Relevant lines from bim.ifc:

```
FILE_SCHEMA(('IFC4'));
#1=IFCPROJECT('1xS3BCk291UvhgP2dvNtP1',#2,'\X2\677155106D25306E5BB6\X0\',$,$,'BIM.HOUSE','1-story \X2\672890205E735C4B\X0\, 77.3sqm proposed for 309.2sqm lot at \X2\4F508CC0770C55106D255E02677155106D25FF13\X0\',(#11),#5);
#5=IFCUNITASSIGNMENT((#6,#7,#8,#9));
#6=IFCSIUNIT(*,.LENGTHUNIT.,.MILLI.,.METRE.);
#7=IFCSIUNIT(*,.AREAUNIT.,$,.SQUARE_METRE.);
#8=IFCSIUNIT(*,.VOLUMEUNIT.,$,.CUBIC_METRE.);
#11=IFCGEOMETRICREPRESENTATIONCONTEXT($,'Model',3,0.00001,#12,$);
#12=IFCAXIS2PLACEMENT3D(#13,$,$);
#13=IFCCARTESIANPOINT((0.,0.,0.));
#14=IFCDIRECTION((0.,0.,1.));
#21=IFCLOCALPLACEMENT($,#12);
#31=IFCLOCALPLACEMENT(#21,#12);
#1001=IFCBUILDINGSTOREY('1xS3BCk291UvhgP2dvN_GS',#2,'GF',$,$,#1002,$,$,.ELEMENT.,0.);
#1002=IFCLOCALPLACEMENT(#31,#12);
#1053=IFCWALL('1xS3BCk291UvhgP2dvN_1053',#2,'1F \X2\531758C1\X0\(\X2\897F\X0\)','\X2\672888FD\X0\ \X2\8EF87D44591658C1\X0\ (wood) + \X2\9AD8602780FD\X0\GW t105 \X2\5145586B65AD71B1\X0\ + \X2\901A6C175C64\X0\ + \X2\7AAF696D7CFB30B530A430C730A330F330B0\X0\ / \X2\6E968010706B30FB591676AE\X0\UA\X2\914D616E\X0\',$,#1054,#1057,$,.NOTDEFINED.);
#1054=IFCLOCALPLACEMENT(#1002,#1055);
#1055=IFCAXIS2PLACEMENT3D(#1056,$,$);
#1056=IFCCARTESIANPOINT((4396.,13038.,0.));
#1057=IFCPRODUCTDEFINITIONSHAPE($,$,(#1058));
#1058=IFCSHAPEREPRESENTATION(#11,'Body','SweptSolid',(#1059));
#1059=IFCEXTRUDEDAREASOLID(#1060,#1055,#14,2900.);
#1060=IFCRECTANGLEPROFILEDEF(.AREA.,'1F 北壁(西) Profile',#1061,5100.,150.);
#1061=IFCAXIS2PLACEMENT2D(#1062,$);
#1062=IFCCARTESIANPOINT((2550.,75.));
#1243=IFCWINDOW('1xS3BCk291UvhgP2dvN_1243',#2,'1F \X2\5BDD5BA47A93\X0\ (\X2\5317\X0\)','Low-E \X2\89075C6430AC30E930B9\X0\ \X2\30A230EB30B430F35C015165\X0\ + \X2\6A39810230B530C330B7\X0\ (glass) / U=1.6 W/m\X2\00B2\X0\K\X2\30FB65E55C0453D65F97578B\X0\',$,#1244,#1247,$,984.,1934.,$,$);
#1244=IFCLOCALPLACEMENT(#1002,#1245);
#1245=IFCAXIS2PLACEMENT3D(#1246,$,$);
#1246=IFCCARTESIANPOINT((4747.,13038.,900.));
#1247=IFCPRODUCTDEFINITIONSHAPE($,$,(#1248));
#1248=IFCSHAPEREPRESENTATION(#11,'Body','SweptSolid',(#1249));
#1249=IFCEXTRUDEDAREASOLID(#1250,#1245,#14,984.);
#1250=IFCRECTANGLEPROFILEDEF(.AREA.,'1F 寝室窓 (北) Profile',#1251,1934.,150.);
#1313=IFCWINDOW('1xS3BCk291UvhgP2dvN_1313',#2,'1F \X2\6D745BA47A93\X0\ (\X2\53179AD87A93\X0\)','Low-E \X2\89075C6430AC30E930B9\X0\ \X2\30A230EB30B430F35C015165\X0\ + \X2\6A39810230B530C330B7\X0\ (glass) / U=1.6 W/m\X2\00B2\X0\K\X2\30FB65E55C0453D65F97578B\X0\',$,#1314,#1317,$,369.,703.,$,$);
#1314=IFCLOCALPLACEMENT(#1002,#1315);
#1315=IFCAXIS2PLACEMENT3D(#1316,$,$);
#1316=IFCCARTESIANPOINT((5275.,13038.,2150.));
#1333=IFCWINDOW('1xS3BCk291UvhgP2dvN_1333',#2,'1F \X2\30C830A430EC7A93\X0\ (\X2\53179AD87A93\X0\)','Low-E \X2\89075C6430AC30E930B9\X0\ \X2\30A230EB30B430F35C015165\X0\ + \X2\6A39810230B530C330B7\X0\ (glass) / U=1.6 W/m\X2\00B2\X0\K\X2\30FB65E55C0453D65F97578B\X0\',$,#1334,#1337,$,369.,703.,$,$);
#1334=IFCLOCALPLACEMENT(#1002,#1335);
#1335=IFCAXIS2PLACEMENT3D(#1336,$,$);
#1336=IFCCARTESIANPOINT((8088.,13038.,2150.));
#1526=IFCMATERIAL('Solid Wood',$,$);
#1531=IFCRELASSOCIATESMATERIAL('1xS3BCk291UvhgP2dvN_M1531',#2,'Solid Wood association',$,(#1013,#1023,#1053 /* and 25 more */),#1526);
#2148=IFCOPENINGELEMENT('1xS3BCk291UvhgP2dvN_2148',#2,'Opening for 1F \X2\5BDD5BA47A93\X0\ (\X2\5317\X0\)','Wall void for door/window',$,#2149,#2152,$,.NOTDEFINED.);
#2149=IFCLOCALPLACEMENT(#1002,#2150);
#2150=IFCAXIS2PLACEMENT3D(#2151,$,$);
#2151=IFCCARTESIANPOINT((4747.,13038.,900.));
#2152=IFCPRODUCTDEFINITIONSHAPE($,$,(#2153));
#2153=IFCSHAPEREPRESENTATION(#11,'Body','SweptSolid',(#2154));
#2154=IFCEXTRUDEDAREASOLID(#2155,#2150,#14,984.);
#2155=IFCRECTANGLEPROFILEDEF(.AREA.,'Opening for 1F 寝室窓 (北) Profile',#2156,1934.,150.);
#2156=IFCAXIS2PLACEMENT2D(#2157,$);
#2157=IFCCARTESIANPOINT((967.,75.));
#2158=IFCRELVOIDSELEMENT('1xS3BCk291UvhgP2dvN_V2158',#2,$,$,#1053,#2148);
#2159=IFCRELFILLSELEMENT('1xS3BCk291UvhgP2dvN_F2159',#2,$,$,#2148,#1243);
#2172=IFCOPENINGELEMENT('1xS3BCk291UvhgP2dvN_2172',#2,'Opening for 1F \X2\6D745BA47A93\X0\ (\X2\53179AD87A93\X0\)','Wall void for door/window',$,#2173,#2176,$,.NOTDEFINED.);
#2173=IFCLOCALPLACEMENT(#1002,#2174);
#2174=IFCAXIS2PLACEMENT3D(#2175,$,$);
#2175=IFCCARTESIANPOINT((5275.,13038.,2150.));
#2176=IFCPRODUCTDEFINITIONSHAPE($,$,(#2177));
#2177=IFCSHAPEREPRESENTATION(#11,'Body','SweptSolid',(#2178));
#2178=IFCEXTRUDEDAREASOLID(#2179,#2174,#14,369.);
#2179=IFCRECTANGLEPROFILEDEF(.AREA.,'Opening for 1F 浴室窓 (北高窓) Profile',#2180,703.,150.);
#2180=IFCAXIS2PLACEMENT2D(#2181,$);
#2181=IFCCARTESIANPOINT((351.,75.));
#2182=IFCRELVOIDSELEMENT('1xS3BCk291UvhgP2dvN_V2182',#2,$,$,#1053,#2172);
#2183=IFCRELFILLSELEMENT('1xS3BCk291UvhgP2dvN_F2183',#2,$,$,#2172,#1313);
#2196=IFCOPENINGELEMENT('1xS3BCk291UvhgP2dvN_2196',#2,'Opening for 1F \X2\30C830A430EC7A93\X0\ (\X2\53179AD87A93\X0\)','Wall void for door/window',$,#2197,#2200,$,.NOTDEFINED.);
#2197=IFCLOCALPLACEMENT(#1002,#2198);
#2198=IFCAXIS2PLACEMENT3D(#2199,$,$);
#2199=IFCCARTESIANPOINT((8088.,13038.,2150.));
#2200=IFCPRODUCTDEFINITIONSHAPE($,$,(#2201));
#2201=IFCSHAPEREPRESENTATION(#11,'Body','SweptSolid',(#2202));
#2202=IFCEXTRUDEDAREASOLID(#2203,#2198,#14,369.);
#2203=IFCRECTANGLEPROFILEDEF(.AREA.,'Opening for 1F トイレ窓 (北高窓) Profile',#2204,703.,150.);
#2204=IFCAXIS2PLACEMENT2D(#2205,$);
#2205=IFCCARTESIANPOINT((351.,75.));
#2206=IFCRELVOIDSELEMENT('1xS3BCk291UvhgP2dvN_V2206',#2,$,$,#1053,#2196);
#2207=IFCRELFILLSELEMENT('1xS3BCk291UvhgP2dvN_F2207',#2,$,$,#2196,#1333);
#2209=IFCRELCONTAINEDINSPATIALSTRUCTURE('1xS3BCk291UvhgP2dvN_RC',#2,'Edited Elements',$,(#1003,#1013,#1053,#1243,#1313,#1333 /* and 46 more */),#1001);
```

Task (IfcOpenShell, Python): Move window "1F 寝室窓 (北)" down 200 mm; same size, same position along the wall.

```python
import numpy as np
import ifcopenshell
import ifcopenshell.api.geometry
import ifcopenshell.util.placement
import ifcopenshell.util.unit

model = ifcopenshell.open("bim.ifc")
unit_scale = ifcopenshell.util.unit.calculate_unit_scale(model)

window = model.by_guid("1xS3BCk291UvhgP2dvN_1243")
opening = window.FillsVoids[0].RelatingOpeningElement
dz = -200.0

shift = np.array([0.0, 0.0, dz])
# The window is not placed relative to its opening, so move both.
for product in (opening, window):
    matrix = ifcopenshell.util.placement.get_local_placement(product.ObjectPlacement)
    matrix[:3, 3] += shift
    ifcopenshell.api.geometry.edit_object_placement(model, product=product, matrix=matrix, is_si=False)

print(f"moved by {dz * unit_scale:+.3f} m")

model.write("bim_rev.ifc")
```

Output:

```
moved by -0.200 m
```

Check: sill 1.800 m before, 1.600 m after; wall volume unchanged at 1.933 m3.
